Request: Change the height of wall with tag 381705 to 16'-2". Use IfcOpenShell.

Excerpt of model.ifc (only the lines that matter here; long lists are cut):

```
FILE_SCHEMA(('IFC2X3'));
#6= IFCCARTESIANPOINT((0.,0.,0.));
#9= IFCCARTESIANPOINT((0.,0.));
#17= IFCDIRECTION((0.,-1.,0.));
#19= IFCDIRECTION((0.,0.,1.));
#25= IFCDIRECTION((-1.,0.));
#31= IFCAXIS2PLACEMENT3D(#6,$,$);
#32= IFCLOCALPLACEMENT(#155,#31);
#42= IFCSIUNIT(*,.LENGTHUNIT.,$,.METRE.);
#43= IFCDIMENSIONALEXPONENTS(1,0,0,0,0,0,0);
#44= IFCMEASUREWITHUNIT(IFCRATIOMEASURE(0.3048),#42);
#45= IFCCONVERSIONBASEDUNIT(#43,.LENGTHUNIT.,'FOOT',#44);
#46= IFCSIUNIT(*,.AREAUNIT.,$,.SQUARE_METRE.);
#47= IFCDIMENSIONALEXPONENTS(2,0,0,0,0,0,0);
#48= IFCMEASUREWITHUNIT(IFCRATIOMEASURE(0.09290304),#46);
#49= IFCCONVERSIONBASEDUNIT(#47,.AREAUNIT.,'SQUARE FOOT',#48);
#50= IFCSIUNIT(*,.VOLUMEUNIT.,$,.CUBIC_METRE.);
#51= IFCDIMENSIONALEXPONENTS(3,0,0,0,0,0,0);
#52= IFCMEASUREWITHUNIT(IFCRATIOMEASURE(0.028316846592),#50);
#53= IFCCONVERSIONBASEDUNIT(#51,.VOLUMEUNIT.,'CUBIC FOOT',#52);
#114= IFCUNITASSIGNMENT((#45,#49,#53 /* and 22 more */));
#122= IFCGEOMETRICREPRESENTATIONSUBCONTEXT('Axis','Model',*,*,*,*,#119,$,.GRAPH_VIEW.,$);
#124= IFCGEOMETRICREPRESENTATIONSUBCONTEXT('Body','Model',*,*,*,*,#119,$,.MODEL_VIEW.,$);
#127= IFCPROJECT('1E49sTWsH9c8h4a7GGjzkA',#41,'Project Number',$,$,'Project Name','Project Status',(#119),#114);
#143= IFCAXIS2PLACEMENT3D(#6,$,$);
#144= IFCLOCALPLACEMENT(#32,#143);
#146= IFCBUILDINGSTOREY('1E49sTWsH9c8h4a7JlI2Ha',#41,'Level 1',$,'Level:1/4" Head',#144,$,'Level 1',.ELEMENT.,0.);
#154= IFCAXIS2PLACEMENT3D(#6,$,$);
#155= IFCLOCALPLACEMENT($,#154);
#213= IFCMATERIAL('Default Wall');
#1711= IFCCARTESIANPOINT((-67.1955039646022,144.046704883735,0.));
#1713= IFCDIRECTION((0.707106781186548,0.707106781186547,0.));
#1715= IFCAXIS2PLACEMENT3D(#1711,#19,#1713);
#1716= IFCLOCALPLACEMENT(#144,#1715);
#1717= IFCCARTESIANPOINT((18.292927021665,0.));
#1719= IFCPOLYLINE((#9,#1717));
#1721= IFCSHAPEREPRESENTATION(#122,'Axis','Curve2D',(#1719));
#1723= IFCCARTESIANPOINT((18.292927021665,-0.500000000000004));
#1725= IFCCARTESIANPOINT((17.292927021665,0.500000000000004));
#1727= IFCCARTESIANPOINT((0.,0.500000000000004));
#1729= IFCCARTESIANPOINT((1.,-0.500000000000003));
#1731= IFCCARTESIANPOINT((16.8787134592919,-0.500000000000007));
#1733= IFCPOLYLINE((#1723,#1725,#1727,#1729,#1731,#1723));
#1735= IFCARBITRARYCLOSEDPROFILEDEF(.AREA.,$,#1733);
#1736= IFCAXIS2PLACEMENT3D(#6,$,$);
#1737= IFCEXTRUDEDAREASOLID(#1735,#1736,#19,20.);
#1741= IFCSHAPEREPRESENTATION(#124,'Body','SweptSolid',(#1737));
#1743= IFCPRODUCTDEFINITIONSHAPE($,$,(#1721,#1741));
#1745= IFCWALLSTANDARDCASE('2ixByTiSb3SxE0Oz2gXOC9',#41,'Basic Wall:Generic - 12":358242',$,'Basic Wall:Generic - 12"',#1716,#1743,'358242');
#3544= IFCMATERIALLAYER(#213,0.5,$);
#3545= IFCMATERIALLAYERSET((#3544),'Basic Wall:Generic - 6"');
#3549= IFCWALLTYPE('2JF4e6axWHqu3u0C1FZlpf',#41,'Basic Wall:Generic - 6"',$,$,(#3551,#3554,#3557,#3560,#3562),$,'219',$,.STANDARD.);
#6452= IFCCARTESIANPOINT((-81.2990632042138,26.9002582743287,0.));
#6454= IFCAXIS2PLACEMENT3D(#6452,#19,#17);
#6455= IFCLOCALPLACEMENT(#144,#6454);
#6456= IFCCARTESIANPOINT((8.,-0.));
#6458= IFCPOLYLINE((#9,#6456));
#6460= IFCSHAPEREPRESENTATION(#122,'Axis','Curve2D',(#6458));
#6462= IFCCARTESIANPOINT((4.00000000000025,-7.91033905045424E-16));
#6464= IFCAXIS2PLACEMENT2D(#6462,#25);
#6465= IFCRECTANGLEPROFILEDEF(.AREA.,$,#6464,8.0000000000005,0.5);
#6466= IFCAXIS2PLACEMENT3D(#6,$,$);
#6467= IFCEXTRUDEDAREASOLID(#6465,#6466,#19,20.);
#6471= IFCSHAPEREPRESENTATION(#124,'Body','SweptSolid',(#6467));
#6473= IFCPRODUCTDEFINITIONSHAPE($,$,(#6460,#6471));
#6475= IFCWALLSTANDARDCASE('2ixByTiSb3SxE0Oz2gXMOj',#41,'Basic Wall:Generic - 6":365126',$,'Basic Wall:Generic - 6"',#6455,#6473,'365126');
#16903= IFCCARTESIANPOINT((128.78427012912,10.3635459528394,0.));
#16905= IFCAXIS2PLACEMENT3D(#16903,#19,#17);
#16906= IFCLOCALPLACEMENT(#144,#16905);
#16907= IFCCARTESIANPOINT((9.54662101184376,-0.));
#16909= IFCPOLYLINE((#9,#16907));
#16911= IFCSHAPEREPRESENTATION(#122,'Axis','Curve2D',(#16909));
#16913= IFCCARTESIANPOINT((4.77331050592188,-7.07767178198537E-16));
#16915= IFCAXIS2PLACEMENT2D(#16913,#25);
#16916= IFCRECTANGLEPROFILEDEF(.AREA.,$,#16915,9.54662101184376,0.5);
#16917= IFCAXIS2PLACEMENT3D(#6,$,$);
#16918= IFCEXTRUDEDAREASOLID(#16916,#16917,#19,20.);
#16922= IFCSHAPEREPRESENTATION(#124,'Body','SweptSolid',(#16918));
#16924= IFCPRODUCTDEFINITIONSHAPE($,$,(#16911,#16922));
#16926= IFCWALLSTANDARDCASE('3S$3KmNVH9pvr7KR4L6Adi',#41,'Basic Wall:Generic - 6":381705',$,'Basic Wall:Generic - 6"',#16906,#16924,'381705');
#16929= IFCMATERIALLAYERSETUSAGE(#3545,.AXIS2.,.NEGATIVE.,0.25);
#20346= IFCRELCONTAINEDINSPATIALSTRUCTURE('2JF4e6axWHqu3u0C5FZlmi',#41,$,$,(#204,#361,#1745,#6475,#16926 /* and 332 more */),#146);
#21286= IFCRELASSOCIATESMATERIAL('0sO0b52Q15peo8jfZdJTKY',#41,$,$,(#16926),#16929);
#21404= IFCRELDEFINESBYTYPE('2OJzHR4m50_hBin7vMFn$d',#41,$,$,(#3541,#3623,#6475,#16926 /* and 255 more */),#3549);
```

```python
import ifcopenshell
import ifcopenshell.geom
import ifcopenshell.util.representation
import ifcopenshell.util.shape
import ifcopenshell.util.unit

model = ifcopenshell.open("model.ifc")
unit_scale = ifcopenshell.util.unit.calculate_unit_scale(model)
settings = ifcopenshell.geom.settings()


def volume(element):
    """Net volume in cubic metres, openings subtracted."""
    shape = ifcopenshell.geom.create_shape(settings, element)
    return ifcopenshell.util.shape.get_volume(shape.geometry)


wall = model.by_guid("3S$3KmNVH9pvr7KR4L6Adi")
before = volume(wall)

body = ifcopenshell.util.representation.get_representation(wall, "Model", "Body")
solid = body.Items[0]
old_height = solid.Depth
solid.Depth = 194 * 0.0254 / unit_scale
after = volume(wall)

print(f"height {old_height:g} -> {solid.Depth:g}, volume {before:.3f} -> {after:.3f} m3")

model.write("model_updated.ifc")
```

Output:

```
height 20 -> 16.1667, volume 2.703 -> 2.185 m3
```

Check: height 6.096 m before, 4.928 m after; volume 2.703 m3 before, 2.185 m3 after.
